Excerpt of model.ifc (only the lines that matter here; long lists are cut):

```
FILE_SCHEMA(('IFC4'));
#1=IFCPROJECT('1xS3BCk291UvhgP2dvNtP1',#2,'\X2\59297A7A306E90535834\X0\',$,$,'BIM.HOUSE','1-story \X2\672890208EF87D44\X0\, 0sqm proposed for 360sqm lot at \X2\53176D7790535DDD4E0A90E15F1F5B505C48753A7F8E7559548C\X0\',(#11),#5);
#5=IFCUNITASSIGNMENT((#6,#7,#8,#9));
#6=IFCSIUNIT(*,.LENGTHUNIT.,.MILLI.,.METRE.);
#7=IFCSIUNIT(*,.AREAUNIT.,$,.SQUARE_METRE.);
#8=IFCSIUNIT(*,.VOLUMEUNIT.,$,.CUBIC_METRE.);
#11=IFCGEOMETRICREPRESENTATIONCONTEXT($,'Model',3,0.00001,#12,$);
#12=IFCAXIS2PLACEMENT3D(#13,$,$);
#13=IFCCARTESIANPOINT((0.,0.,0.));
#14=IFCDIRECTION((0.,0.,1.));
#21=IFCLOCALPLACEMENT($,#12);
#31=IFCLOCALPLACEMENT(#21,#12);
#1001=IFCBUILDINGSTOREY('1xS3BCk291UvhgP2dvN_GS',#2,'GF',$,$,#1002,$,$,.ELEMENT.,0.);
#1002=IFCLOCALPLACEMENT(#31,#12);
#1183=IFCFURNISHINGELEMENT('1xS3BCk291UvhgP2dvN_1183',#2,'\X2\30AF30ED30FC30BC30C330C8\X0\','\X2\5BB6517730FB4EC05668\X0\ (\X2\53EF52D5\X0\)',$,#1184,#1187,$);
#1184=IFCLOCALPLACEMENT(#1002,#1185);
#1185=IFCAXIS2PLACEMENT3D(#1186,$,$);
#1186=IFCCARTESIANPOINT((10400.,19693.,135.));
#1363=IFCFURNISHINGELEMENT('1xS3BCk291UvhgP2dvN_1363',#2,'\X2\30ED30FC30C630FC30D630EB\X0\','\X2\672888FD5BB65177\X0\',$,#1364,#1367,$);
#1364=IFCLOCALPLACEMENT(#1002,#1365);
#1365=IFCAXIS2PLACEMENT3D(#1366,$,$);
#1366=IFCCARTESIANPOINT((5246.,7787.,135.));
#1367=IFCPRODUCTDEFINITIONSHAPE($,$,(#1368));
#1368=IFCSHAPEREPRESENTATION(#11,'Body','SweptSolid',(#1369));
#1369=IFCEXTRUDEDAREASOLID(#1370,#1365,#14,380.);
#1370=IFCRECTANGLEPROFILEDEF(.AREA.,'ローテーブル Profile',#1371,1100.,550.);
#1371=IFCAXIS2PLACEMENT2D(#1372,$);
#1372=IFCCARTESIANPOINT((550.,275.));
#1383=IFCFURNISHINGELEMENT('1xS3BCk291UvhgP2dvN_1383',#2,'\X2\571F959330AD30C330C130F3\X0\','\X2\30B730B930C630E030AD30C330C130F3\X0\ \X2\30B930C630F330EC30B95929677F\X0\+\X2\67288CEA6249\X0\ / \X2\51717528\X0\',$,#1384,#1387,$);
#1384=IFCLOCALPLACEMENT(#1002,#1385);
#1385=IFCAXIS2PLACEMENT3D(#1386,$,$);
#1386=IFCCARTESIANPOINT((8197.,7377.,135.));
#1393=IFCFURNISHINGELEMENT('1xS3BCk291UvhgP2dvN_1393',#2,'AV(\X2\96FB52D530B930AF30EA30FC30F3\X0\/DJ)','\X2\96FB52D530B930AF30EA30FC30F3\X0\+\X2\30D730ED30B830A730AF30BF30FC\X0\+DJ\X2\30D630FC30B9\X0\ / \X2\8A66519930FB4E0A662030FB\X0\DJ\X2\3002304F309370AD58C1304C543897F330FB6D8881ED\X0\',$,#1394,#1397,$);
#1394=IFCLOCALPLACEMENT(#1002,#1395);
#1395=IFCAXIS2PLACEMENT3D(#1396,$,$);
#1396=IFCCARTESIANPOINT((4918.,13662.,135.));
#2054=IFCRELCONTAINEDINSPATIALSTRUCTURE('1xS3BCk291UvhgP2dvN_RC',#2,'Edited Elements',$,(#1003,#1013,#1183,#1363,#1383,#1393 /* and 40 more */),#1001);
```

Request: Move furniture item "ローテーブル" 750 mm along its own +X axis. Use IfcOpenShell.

```python
import ifcopenshell
import ifcopenshell.api.geometry
import ifcopenshell.util.placement

model = ifcopenshell.open("model.ifc")

item = model.by_guid("1xS3BCk291UvhgP2dvN_1363")
matrix = ifcopenshell.util.placement.get_local_placement(item.ObjectPlacement)
matrix[:3, 3] += matrix[:3, 0] * 750.0
ifcopenshell.api.geometry.edit_object_placement(model, product=item, matrix=matrix, is_si=False)

print(ifcopenshell.util.placement.get_local_placement(item.ObjectPlacement).round(3) + 0.0)

model.write("model_updated.ifc")
```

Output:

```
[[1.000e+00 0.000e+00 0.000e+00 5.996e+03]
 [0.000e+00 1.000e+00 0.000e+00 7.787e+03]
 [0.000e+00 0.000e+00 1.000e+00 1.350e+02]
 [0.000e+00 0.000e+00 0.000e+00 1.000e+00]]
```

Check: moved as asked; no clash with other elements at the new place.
